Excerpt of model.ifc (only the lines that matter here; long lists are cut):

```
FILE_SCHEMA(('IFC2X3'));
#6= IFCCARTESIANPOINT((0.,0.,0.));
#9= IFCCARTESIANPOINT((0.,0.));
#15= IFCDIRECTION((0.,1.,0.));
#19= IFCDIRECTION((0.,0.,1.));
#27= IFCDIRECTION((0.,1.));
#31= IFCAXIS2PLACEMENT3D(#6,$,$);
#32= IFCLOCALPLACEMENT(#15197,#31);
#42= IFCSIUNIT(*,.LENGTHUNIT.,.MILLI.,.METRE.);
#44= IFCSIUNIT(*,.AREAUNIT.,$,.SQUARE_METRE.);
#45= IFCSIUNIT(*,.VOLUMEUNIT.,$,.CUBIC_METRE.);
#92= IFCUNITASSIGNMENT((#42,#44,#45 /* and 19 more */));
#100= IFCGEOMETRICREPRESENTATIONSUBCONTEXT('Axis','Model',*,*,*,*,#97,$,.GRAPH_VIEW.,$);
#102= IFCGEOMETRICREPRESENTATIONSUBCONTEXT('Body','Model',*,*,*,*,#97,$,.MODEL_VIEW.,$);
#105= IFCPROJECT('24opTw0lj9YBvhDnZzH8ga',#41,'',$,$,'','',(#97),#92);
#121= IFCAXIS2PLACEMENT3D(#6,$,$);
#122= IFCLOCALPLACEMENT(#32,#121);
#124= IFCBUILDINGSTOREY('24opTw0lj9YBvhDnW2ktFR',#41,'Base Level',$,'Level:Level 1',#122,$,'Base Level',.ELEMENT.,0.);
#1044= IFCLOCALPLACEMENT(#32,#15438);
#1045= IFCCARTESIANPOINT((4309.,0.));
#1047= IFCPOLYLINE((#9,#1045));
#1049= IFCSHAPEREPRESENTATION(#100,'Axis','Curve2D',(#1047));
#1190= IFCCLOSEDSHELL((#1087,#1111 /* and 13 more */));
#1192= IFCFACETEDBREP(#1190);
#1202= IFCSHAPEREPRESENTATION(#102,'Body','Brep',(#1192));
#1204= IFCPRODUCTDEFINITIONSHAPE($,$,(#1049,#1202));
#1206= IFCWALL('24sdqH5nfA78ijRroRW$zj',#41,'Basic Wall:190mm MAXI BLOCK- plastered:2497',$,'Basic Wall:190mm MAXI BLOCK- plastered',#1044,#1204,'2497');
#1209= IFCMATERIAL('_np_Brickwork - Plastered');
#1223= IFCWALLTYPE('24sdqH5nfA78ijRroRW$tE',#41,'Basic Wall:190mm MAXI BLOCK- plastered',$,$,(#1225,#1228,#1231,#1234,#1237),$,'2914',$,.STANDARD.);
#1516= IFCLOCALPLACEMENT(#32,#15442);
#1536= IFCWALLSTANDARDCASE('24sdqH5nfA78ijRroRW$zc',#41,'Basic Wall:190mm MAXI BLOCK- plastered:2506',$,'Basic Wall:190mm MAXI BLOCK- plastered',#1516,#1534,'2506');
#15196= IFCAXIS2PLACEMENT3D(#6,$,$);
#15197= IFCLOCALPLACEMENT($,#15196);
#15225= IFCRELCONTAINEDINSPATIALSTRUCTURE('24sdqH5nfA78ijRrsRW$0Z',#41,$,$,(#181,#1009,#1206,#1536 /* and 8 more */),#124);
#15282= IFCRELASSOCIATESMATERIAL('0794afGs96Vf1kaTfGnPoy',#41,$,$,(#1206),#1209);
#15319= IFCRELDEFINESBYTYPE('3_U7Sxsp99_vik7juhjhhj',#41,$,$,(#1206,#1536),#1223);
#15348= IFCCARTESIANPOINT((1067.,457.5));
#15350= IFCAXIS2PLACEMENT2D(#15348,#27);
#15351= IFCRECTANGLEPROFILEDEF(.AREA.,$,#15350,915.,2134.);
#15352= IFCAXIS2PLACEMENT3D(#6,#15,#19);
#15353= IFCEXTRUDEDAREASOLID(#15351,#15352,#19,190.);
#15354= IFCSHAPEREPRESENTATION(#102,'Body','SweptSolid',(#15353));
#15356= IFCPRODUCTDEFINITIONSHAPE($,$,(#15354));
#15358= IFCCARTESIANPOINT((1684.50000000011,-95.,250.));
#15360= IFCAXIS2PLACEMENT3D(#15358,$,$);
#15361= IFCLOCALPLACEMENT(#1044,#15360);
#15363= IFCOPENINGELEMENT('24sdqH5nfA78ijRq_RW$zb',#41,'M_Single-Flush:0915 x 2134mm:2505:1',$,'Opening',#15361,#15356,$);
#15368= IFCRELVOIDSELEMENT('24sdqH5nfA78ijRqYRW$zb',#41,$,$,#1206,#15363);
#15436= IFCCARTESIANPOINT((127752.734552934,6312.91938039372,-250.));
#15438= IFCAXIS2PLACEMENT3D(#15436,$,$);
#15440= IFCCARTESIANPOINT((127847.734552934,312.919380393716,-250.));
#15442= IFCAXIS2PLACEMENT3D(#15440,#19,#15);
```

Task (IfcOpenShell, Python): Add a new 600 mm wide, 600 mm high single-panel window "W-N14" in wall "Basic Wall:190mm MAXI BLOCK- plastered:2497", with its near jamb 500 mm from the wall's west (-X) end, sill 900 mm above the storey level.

```python
import numpy as np
import ifcopenshell
import ifcopenshell.api.feature
import ifcopenshell.api.geometry
import ifcopenshell.api.root
import ifcopenshell.api.spatial
import ifcopenshell.api.type
import ifcopenshell.geom
import ifcopenshell.util.element
import ifcopenshell.util.placement
import ifcopenshell.util.representation
import ifcopenshell.util.shape
import ifcopenshell.util.unit

model = ifcopenshell.open("model.ifc")
unit_scale = ifcopenshell.util.unit.calculate_unit_scale(model)
settings = ifcopenshell.geom.settings()


def volume(element):
    """Net volume in cubic metres, openings subtracted."""
    shape = ifcopenshell.geom.create_shape(settings, element)
    return ifcopenshell.util.shape.get_volume(shape.geometry)


wall = model.by_guid("24sdqH5nfA78ijRroRW$zj")
storey = ifcopenshell.util.element.get_container(wall, ifc_class="IfcBuildingStorey")
context = ifcopenshell.util.representation.get_context(model, "Model", "Body", "MODEL_VIEW")
before = volume(wall)

width, height, from_end, sill = 0.6, 0.6, 0.5, 0.9  # metres

# The wall runs along its own X axis, and the end named is its -X end.
wall_shape = ifcopenshell.geom.create_shape(settings, wall)
x, y, z = ifcopenshell.util.shape.get_vertices(wall_shape.geometry).T
start = x.min() + from_end
face, thickness = float(y.min()), float(y.max() - y.min())
wall_matrix = ifcopenshell.util.placement.get_local_placement(wall.ObjectPlacement)
level = ifcopenshell.util.placement.get_local_placement(storey.ObjectPlacement)[2, 3]


def in_wall(x, y):
    """Placement at x, y metres in the wall's axes, at sill height."""
    matrix = wall_matrix.copy()
    matrix[:, 3] = wall_matrix @ np.array([x / unit_scale, y / unit_scale, 0.0, 1.0])
    matrix[2, 3] = level + sill / unit_scale
    return matrix


# Opening: a box that overshoots both wall faces by 50 mm.
opening = ifcopenshell.api.root.create_entity(model, ifc_class="IfcOpeningElement")
box = ifcopenshell.api.geometry.add_wall_representation(
    model, context=context, length=width, height=height, thickness=thickness + 0.1
)
ifcopenshell.api.geometry.assign_representation(model, product=opening, representation=box)
ifcopenshell.api.geometry.edit_object_placement(model, product=opening, matrix=in_wall(start, face - 0.05), is_si=False)
ifcopenshell.api.feature.add_feature(model, feature=opening, element=wall)

window = ifcopenshell.api.root.create_entity(model, ifc_class="IfcWindow", name="W-N14")
window.OverallWidth, window.OverallHeight = width / unit_scale, height / unit_scale
body = ifcopenshell.api.geometry.add_window_representation(
    model,
    context=context,
    overall_width=window.OverallWidth,
    overall_height=window.OverallHeight,
    partition_type="SINGLE_PANEL",
)
ifcopenshell.api.geometry.assign_representation(model, product=window, representation=body)
ifcopenshell.api.spatial.assign_container(model, products=[window], relating_structure=storey)
fills = ifcopenshell.api.feature.add_filling(model, opening=opening, element=window)
fills.OwnerHistory = window.OwnerHistory  # required in IFC2X3

# IFC2X3 keeps the operation on the window style.
style = ifcopenshell.api.root.create_entity(model, ifc_class="IfcWindowStyle", name="W-N14")
style.OperationType, style.ConstructionType = "SINGLE_PANEL", "NOTDEFINED"
style.ParameterTakesPrecedence = style.Sizeable = False
ifcopenshell.api.type.assign_type(model, related_objects=[window], relating_type=style)

# Centre the window in the wall's thickness.
ifcopenshell.api.geometry.edit_object_placement(model, product=window, matrix=in_wall(start, face), is_si=False)
window_shape = ifcopenshell.geom.create_shape(settings, window)
depth = ifcopenshell.util.shape.get_vertices(window_shape.geometry)[:, 1]
offset = face + thickness / 2 - (depth.min() + depth.max()) / 2
ifcopenshell.api.geometry.edit_object_placement(model, product=window, matrix=in_wall(start, offset), is_si=False)

after = volume(wall)

print(f"wall volume {before:.3f} -> {after:.3f} m3")

model.write("model_rev.ifc")
```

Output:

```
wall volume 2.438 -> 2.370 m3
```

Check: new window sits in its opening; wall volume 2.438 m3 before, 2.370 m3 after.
